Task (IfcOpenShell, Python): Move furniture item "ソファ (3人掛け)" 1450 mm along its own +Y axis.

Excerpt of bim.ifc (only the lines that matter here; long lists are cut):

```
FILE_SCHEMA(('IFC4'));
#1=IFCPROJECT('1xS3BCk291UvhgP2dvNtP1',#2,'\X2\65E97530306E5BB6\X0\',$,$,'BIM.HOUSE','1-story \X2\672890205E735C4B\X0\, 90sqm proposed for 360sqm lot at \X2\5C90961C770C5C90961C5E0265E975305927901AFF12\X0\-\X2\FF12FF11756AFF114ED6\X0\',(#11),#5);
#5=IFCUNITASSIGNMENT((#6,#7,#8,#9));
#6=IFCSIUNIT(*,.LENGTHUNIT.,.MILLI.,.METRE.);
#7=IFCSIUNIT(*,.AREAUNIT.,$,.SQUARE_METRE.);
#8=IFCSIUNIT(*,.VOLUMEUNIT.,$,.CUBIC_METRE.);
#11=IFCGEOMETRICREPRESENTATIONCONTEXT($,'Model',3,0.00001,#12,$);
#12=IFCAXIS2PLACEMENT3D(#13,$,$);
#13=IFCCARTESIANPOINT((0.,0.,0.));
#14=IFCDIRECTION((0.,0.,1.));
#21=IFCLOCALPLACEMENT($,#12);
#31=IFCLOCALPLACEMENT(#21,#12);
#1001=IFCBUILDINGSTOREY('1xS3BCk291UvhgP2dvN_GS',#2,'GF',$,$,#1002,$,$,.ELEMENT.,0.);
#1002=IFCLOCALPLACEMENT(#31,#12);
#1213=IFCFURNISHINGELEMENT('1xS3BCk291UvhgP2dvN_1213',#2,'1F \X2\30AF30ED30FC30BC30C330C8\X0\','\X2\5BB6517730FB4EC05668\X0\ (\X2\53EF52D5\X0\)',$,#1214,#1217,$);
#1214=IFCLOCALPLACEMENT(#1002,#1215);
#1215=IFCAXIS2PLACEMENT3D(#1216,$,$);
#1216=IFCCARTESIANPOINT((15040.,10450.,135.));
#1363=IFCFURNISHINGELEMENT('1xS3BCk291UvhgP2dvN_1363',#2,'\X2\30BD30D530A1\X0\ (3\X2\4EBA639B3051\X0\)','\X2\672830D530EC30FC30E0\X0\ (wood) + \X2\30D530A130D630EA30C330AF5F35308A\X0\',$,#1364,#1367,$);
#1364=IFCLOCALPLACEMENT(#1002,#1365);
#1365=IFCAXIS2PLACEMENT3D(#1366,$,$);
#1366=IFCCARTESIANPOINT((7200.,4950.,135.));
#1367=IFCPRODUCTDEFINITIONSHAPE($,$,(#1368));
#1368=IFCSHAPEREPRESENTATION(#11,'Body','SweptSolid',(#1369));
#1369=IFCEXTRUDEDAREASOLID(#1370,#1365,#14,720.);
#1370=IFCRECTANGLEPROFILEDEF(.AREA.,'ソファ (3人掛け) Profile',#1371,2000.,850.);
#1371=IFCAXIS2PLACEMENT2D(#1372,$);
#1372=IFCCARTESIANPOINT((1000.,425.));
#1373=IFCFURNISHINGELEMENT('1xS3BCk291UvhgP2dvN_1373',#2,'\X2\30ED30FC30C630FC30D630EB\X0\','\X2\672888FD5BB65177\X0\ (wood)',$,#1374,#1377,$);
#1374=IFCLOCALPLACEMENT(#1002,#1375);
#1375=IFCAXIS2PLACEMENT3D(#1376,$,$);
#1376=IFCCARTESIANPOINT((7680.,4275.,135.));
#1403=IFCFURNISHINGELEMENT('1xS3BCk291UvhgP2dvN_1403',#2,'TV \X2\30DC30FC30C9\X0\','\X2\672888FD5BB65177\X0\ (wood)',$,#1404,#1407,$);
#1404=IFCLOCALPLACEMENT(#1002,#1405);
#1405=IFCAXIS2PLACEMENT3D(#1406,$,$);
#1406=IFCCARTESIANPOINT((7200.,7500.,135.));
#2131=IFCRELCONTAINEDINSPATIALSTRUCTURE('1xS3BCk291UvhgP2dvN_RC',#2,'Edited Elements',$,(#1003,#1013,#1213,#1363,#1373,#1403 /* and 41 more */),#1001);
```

```python
import ifcopenshell
import ifcopenshell.api.geometry
import ifcopenshell.util.placement

model = ifcopenshell.open("bim.ifc")

item = model.by_guid("1xS3BCk291UvhgP2dvN_1363")
matrix = ifcopenshell.util.placement.get_local_placement(item.ObjectPlacement)
matrix[:3, 3] += matrix[:3, 1] * 1450.0
ifcopenshell.api.geometry.edit_object_placement(model, product=item, matrix=matrix, is_si=False)

print(ifcopenshell.util.placement.get_local_placement(item.ObjectPlacement).round(3) + 0.0)

model.write("bim_v2.ifc")
```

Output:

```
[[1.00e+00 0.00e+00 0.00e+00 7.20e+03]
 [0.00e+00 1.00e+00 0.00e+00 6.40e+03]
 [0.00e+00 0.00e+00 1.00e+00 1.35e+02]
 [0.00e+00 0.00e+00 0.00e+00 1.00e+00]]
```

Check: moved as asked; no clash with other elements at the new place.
